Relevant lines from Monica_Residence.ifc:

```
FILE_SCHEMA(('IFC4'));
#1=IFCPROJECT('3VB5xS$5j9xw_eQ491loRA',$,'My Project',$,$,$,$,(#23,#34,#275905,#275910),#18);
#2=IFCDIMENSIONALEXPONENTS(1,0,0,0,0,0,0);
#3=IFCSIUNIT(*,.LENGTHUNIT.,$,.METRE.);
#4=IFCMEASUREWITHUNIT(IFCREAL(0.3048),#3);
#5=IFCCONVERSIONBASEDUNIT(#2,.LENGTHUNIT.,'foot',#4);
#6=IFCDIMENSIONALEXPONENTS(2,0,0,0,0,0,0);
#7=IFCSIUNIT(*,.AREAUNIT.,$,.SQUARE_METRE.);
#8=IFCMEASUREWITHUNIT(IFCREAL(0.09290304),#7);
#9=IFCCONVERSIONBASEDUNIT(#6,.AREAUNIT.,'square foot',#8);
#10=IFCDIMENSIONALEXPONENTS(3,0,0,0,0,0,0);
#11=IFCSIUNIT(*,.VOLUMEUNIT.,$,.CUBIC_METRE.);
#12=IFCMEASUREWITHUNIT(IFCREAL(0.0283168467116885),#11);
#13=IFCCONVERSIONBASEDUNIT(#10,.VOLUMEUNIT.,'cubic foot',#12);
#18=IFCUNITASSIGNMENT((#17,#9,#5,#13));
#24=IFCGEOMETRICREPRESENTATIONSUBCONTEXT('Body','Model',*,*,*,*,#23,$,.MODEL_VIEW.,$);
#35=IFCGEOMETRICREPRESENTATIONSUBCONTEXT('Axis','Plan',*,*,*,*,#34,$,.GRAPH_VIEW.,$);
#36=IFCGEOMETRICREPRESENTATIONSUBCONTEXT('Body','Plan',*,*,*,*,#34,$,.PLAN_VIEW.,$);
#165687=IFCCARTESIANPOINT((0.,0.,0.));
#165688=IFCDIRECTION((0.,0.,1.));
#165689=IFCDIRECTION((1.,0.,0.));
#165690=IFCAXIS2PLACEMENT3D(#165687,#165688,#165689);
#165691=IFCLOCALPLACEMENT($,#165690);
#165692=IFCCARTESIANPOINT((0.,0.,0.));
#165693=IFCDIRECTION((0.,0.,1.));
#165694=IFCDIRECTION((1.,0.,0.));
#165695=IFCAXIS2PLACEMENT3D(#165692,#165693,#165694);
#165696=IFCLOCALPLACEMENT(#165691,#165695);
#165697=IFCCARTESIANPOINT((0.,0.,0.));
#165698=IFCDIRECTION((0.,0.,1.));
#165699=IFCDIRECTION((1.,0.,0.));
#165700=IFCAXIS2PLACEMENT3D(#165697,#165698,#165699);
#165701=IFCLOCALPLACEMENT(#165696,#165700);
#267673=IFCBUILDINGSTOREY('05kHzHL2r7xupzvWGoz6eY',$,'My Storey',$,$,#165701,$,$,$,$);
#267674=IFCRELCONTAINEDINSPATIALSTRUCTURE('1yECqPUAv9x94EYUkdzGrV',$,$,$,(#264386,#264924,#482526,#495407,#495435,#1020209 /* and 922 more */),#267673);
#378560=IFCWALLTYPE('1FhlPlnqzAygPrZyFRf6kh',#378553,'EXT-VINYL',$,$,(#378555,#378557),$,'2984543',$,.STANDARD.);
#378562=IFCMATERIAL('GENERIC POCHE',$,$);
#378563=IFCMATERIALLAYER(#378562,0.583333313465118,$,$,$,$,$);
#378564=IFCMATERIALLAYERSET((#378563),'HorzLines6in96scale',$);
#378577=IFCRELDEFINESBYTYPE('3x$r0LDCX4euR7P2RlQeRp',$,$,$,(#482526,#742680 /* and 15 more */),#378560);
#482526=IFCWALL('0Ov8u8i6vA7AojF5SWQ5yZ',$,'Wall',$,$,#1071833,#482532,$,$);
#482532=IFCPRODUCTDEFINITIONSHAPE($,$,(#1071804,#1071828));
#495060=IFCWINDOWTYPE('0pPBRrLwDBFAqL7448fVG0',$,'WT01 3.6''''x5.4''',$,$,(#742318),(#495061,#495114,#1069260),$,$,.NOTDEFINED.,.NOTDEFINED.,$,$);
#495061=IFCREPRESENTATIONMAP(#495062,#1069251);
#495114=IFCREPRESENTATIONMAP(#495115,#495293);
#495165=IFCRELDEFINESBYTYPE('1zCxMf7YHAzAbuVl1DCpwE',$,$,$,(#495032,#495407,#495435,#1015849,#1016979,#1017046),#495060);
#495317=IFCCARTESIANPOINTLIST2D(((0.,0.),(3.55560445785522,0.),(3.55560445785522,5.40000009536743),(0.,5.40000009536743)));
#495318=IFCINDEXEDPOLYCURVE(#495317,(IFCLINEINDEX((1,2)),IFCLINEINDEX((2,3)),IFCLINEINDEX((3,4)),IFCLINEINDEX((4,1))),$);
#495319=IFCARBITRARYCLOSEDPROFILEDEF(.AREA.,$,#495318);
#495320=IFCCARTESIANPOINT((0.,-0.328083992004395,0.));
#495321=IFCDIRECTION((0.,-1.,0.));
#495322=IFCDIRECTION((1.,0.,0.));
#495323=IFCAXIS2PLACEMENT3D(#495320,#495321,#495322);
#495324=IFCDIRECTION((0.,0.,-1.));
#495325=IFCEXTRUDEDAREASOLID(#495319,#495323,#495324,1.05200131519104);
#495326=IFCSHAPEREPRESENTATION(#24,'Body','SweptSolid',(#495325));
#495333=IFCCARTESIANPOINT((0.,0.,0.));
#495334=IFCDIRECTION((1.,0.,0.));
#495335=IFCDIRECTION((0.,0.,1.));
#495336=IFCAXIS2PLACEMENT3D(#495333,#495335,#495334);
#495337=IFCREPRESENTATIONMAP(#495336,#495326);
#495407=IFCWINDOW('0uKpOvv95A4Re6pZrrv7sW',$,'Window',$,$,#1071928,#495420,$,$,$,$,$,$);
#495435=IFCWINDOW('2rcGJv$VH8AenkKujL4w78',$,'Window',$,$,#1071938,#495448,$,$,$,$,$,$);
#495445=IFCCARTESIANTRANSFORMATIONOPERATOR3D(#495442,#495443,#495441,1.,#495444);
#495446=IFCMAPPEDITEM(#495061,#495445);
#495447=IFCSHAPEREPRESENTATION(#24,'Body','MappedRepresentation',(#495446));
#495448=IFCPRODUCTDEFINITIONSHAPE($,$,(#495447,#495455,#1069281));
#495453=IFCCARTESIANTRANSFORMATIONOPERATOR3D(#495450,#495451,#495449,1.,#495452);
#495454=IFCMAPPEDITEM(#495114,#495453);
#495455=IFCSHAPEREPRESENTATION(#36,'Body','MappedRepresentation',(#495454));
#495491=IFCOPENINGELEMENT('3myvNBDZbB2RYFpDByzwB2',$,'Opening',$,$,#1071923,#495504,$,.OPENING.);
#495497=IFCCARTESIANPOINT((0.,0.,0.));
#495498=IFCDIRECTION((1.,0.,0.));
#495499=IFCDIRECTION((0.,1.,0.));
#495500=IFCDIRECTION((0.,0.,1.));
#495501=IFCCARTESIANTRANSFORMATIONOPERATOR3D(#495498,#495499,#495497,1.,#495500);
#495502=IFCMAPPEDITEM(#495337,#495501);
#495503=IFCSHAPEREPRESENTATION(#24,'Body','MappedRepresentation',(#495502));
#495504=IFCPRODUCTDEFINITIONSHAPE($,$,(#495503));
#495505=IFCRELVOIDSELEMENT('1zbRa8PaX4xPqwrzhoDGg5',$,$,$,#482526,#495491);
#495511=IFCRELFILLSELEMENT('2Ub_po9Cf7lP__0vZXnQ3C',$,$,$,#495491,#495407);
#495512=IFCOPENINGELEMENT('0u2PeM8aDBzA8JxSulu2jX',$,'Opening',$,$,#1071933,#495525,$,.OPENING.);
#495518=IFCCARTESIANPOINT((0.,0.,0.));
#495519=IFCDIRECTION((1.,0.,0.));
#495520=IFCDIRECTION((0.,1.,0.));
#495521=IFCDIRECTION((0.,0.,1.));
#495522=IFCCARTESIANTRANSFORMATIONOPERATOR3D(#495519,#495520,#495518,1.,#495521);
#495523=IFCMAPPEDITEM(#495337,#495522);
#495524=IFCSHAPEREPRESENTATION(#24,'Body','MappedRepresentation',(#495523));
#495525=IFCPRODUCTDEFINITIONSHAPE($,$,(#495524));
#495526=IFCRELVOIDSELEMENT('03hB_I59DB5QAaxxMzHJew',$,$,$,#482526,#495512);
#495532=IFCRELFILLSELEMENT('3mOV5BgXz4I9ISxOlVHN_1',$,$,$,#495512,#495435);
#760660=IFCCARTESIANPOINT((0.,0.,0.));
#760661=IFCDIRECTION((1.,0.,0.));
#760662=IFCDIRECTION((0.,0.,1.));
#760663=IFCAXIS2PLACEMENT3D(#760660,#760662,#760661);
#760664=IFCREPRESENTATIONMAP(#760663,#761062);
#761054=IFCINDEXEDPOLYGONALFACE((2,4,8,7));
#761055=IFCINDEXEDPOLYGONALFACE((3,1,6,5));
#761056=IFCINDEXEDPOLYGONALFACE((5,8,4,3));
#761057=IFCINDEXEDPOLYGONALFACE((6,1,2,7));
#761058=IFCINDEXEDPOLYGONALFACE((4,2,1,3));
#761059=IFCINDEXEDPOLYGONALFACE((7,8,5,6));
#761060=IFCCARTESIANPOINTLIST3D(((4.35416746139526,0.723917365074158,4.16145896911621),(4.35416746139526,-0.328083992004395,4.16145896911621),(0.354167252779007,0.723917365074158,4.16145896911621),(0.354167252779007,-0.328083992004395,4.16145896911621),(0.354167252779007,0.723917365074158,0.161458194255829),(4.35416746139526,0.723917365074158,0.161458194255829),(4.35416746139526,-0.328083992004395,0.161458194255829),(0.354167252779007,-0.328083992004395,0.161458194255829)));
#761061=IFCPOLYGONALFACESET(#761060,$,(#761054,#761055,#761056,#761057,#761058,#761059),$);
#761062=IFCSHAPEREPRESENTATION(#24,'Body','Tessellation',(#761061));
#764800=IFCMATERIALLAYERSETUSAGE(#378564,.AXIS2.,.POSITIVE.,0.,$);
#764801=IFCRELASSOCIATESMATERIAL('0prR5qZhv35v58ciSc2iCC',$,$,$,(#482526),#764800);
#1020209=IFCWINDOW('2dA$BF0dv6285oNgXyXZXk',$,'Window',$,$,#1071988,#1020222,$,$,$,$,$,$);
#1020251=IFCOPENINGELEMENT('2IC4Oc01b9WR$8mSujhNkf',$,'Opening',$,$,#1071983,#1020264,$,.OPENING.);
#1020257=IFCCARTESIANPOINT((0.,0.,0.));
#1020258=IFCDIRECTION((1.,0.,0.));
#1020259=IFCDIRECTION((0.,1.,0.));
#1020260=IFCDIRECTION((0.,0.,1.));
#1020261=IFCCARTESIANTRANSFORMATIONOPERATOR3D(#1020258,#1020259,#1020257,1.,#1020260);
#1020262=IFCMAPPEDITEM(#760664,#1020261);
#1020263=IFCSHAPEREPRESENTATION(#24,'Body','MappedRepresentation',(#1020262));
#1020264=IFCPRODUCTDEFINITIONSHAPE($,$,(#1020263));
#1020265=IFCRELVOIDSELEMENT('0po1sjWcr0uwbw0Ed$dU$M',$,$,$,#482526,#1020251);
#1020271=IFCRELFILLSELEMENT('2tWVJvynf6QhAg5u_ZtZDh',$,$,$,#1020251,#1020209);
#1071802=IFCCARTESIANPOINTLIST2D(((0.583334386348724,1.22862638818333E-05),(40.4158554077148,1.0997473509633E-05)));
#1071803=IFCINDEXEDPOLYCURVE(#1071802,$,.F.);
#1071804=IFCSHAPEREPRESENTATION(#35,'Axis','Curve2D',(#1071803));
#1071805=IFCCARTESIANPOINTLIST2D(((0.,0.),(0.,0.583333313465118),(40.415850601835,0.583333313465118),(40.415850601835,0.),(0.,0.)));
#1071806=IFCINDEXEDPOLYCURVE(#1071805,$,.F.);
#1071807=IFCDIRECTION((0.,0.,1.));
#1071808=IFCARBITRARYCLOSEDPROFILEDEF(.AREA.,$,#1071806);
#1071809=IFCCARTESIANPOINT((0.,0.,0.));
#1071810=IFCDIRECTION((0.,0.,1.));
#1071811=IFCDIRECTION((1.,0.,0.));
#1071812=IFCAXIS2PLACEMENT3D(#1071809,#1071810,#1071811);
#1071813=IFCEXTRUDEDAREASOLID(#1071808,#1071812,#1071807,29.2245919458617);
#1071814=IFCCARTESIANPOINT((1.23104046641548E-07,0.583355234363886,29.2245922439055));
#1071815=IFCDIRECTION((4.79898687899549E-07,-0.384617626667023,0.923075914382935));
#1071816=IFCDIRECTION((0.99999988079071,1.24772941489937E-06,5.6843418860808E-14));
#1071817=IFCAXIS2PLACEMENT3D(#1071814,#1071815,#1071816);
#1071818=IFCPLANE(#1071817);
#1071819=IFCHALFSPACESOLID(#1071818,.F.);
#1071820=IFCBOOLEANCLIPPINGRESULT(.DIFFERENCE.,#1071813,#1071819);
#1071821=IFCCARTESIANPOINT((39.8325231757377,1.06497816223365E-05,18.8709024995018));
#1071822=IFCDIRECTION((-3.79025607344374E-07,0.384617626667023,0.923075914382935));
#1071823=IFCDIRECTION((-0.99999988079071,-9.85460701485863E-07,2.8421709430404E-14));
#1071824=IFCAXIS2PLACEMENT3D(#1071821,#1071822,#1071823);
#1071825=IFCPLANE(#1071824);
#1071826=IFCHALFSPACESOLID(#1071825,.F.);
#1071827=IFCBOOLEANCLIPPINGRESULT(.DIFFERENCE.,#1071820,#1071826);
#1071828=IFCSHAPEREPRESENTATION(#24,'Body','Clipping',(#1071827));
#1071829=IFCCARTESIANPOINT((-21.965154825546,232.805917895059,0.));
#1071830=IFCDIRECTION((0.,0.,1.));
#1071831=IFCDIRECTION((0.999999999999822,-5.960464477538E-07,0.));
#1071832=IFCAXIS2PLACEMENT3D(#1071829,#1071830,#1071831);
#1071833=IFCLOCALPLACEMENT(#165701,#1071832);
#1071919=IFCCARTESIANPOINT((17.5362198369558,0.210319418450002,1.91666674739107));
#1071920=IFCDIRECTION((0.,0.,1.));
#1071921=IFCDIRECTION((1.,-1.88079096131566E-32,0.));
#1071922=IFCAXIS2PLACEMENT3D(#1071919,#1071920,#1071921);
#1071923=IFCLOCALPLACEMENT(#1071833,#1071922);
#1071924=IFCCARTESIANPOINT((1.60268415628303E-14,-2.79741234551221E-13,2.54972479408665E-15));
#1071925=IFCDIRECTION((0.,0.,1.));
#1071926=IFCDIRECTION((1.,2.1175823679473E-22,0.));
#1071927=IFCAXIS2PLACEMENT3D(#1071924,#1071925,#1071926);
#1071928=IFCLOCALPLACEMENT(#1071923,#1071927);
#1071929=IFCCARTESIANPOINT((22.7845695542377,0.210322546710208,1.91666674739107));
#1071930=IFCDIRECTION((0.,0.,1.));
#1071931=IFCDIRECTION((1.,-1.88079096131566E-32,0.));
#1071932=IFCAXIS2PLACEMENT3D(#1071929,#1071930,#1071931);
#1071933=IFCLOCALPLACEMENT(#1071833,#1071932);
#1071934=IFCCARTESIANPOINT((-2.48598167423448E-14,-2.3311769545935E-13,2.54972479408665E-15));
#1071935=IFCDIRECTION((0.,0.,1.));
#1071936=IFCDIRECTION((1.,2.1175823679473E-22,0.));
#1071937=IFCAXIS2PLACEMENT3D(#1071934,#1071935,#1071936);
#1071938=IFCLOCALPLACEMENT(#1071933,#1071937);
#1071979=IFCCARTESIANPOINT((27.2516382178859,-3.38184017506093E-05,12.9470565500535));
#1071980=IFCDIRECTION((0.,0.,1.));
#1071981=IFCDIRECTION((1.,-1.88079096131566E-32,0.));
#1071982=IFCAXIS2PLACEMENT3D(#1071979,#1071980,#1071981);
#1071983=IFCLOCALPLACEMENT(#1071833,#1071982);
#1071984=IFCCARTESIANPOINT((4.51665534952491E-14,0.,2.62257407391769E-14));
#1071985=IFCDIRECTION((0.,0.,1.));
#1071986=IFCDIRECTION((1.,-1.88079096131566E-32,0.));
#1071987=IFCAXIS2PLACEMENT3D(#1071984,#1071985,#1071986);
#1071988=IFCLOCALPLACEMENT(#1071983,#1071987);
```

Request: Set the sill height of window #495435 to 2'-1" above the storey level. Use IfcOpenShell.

```python
import numpy as np
import ifcopenshell
import ifcopenshell.api.geometry
import ifcopenshell.geom
import ifcopenshell.util.element
import ifcopenshell.util.placement
import ifcopenshell.util.shape
import ifcopenshell.util.unit

model = ifcopenshell.open("Monica_Residence.ifc")
unit_scale = ifcopenshell.util.unit.calculate_unit_scale(model)

window = model.by_id(495435)
opening = window.FillsVoids[0].RelatingOpeningElement
storey = ifcopenshell.util.element.get_container(window, ifc_class="IfcBuildingStorey")
level = ifcopenshell.util.placement.get_local_placement(storey.ObjectPlacement)[2, 3]

# The opening's origin need not be at the sill, so measure its lowest point.
shape = ifcopenshell.geom.create_shape(ifcopenshell.geom.settings(), opening)
bottom = ifcopenshell.util.shape.get_shape_bottom_elevation(shape, shape.geometry) / unit_scale
dz = level + 25 * 0.0254 / unit_scale - bottom

shift = np.array([0.0, 0.0, dz])
# The window is placed relative to its opening, so it follows when the opening moves.
matrix = ifcopenshell.util.placement.get_local_placement(opening.ObjectPlacement)
matrix[:3, 3] += shift
ifcopenshell.api.geometry.edit_object_placement(
    model, product=opening, matrix=matrix, is_si=False, should_transform_children=True
)

print(f"moved by {dz * unit_scale:+.3f} m")

model.write("Monica_Residence_updated.ifc")
```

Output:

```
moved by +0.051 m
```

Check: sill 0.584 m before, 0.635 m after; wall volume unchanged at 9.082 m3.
